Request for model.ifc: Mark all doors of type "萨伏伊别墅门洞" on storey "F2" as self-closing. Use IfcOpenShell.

First a look at what the model holds.

```python
import ifcopenshell
import ifcopenshell.util.element

model = ifcopenshell.open("model.ifc")
print(model.schema)
storey = next(s for s in model.by_type("IfcBuildingStorey") if s.Name == "F2")
doors = [e for e in ifcopenshell.util.element.get_decomposition(storey) if e.is_a("IfcDoor")]
seen = {}
for e in doors:
    element_type = ifcopenshell.util.element.get_type(e)
    key = (element_type.Name if element_type != e and element_type else None, ifcopenshell.util.element.get_pset(e, "Pset_DoorCommon", "SelfClosing"))
    seen[key] = seen.get(key, 0) + 1
for (name, value), count in sorted(seen.items(), key=str):
    print(count, "x", name, "|", value)
```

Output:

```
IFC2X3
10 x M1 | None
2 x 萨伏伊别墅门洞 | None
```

```python
import ifcopenshell
import ifcopenshell.api.pset
import ifcopenshell.util.element

model = ifcopenshell.open("model.ifc")

storey = next(s for s in model.by_type("IfcBuildingStorey") if s.Name == "F2")
doors = [e for e in ifcopenshell.util.element.get_decomposition(storey) if e.is_a("IfcDoor")]

count = 0
for e in doors:
    element_type = ifcopenshell.util.element.get_type(e)
    if element_type in (None, e) or element_type.Name != "萨伏伊别墅门洞":
        continue
    # add_pset returns the element's existing set when there is one.
    pset = ifcopenshell.api.pset.add_pset(model, product=e, name="Pset_DoorCommon")
    ifcopenshell.api.pset.edit_pset(model, pset=pset, properties={"SelfClosing": True})
    count += 1

print(count, "doors updated")

model.write("model_edited.ifc")
```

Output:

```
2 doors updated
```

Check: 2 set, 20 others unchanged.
